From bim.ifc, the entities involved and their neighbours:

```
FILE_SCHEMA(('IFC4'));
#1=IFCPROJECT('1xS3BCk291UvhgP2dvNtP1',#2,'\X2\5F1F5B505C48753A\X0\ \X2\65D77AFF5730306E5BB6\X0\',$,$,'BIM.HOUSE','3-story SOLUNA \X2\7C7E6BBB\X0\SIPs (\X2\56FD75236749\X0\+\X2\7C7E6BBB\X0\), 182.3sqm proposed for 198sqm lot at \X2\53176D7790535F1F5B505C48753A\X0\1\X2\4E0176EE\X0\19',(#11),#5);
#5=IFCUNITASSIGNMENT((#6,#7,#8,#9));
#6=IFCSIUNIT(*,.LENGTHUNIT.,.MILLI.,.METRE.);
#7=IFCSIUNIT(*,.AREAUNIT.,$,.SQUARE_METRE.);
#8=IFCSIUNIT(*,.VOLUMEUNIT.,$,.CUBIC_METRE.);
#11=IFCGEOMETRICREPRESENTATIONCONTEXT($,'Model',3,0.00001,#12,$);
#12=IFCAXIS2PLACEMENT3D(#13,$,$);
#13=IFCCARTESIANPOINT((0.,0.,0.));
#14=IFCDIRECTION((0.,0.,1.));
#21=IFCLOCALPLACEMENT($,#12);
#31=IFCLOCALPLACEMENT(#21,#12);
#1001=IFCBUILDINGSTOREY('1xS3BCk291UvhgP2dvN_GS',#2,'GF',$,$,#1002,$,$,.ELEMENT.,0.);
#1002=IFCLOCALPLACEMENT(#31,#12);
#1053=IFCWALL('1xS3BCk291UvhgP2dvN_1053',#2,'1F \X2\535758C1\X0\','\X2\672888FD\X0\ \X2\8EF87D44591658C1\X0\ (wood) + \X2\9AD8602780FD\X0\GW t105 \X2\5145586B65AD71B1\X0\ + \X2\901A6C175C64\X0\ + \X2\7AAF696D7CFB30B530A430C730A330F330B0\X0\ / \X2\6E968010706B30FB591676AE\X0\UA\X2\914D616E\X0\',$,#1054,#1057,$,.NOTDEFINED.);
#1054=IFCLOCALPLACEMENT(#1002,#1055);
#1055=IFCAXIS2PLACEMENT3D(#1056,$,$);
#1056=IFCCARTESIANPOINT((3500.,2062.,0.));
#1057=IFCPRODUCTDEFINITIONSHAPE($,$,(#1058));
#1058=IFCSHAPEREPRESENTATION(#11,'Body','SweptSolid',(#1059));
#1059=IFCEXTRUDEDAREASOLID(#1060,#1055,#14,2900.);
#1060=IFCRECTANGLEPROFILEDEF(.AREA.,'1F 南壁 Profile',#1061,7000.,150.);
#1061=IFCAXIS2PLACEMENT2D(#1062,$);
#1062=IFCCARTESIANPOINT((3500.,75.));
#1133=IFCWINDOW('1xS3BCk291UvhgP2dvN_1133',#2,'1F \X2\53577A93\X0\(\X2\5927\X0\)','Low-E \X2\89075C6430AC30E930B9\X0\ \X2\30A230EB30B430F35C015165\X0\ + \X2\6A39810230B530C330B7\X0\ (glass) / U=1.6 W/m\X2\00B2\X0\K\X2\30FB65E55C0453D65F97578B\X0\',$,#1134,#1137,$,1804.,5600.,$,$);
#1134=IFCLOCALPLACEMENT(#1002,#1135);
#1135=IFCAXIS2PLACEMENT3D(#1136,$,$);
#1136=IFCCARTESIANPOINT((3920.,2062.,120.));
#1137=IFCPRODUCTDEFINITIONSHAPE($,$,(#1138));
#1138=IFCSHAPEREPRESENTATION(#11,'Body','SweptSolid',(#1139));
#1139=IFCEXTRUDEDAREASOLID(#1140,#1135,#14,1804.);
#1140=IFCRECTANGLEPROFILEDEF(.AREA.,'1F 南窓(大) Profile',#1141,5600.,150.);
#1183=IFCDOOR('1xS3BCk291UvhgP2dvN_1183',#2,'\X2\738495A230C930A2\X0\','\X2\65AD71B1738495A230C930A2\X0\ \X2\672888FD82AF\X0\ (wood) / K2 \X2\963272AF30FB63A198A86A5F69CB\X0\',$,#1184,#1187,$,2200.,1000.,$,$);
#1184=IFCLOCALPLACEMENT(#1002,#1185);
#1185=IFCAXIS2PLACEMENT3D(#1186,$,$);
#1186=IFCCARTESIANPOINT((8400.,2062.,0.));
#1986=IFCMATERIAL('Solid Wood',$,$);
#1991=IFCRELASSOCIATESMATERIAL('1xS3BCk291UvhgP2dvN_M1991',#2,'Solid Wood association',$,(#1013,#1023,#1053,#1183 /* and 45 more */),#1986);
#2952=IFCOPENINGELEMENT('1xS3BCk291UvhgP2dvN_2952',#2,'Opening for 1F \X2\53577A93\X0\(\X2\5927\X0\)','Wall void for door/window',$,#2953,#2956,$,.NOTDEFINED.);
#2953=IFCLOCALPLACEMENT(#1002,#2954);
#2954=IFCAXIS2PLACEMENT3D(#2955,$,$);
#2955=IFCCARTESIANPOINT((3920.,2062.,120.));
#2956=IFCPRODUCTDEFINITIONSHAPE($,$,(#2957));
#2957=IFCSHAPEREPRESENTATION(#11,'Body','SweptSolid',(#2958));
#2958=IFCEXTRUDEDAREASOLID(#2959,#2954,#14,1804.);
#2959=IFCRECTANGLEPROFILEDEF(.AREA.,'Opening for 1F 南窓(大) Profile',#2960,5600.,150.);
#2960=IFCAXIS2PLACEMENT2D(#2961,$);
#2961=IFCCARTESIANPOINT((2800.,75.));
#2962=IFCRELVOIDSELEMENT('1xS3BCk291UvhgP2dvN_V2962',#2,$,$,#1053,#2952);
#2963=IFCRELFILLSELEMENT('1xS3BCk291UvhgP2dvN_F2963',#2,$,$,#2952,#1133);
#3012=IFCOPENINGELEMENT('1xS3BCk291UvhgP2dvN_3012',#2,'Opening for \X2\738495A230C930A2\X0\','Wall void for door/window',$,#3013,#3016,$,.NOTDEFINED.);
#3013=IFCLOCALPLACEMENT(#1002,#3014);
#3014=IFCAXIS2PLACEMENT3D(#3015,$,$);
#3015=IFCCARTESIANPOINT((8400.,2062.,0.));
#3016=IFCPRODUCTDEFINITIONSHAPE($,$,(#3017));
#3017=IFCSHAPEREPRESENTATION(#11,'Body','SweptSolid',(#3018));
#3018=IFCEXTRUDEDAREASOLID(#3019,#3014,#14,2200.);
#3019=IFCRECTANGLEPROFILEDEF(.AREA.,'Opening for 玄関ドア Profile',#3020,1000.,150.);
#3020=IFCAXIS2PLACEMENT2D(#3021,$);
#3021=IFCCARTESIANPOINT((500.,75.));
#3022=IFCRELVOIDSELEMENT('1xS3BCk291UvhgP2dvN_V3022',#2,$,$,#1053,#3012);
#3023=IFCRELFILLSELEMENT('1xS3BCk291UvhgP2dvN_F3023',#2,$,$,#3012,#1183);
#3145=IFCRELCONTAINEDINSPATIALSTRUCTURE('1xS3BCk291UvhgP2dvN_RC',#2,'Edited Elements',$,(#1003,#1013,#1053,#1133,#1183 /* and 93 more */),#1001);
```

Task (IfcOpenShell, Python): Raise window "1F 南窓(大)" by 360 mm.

```python
import numpy as np
import ifcopenshell
import ifcopenshell.api.geometry
import ifcopenshell.util.placement
import ifcopenshell.util.unit

model = ifcopenshell.open("bim.ifc")
unit_scale = ifcopenshell.util.unit.calculate_unit_scale(model)

window = model.by_guid("1xS3BCk291UvhgP2dvN_1133")
opening = window.FillsVoids[0].RelatingOpeningElement
dz = 360.0

shift = np.array([0.0, 0.0, dz])
# The window is not placed relative to its opening, so move both.
for product in (opening, window):
    matrix = ifcopenshell.util.placement.get_local_placement(product.ObjectPlacement)
    matrix[:3, 3] += shift
    ifcopenshell.api.geometry.edit_object_placement(model, product=product, matrix=matrix, is_si=False)

print(f"moved by {dz * unit_scale:+.3f} m")

model.write("bim_rev.ifc")
```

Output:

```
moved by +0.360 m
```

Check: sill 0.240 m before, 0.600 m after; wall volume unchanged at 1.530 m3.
